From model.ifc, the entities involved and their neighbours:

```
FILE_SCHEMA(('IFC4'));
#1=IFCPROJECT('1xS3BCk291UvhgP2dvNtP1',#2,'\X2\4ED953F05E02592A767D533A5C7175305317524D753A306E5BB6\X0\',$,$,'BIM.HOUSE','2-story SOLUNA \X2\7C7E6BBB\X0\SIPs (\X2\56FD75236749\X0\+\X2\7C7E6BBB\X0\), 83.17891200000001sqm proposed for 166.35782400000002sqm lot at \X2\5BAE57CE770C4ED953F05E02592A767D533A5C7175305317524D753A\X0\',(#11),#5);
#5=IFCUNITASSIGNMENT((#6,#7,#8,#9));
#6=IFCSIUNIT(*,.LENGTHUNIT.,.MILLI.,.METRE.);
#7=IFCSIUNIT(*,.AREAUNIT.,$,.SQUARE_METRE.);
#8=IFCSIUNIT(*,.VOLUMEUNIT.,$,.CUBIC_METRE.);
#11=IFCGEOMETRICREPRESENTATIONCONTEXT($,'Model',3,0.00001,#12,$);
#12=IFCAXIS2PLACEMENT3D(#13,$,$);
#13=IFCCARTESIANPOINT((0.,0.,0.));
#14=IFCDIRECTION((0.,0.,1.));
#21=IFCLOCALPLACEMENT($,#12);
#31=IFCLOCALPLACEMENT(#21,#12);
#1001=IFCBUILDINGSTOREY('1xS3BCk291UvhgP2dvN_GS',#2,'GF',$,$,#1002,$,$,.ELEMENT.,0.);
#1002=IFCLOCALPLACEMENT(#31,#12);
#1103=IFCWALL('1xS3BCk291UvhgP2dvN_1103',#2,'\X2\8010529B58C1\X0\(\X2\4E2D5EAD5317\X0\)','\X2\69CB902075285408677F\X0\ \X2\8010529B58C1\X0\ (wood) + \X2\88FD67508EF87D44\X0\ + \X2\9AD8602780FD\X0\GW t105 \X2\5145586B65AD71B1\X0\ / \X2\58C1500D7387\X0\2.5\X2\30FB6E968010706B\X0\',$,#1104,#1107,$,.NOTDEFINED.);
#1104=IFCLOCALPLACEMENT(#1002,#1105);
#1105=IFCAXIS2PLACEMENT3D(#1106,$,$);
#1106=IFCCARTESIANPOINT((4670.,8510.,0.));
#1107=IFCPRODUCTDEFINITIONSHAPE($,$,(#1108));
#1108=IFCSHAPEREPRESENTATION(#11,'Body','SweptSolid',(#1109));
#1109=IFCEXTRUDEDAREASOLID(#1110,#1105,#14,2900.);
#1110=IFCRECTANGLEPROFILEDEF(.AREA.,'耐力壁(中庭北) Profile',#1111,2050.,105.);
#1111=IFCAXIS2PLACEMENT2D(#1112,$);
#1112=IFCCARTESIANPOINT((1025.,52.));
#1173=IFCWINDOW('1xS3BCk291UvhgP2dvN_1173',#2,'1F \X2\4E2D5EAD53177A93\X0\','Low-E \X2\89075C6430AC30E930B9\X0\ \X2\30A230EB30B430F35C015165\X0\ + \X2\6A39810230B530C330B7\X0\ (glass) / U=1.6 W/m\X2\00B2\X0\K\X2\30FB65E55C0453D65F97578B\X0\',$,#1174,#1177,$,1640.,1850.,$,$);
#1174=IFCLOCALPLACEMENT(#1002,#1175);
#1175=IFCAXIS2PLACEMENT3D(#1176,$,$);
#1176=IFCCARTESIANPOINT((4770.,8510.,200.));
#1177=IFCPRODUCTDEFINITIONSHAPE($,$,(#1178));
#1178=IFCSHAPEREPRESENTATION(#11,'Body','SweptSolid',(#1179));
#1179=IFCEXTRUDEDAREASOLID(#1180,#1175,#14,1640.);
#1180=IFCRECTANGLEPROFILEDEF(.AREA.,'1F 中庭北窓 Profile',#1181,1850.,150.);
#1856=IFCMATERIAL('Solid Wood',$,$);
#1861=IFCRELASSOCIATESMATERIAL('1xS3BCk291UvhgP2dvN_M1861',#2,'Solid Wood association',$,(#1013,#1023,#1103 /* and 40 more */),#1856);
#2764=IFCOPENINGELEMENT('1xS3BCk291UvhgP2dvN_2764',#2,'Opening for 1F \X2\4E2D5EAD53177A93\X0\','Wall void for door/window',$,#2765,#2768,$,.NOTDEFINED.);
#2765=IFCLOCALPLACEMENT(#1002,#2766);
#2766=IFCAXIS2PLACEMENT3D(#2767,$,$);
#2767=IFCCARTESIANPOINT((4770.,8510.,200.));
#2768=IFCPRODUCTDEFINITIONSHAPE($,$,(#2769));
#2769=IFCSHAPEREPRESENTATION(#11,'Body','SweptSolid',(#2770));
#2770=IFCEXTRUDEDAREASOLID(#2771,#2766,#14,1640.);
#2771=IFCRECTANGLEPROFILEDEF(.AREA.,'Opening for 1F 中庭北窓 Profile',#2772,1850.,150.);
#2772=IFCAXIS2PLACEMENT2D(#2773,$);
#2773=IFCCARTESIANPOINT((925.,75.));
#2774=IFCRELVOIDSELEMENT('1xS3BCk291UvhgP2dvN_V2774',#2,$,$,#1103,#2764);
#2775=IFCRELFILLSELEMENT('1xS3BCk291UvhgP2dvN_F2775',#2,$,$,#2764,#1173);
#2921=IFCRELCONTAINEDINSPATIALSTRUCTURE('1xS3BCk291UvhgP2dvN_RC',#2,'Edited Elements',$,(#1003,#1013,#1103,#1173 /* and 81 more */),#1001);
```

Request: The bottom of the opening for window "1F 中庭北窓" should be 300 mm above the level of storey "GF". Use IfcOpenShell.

```python
import numpy as np
import ifcopenshell
import ifcopenshell.api.geometry
import ifcopenshell.geom
import ifcopenshell.util.element
import ifcopenshell.util.placement
import ifcopenshell.util.shape
import ifcopenshell.util.unit

model = ifcopenshell.open("model.ifc")
unit_scale = ifcopenshell.util.unit.calculate_unit_scale(model)

window = model.by_guid("1xS3BCk291UvhgP2dvN_1173")
opening = window.FillsVoids[0].RelatingOpeningElement
storey = ifcopenshell.util.element.get_container(window, ifc_class="IfcBuildingStorey")
level = ifcopenshell.util.placement.get_local_placement(storey.ObjectPlacement)[2, 3]

# The opening's origin need not be at the sill, so measure its lowest point.
shape = ifcopenshell.geom.create_shape(ifcopenshell.geom.settings(), opening)
bottom = ifcopenshell.util.shape.get_shape_bottom_elevation(shape, shape.geometry) / unit_scale
dz = level + 0.3 / unit_scale - bottom

shift = np.array([0.0, 0.0, dz])
# The window is not placed relative to its opening, so move both.
for product in (opening, window):
    matrix = ifcopenshell.util.placement.get_local_placement(product.ObjectPlacement)
    matrix[:3, 3] += shift
    ifcopenshell.api.geometry.edit_object_placement(model, product=product, matrix=matrix, is_si=False)

print(f"moved by {dz * unit_scale:+.3f} m")

model.write("model_v2.ifc")
```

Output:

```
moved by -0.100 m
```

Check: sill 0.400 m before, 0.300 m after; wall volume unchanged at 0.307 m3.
